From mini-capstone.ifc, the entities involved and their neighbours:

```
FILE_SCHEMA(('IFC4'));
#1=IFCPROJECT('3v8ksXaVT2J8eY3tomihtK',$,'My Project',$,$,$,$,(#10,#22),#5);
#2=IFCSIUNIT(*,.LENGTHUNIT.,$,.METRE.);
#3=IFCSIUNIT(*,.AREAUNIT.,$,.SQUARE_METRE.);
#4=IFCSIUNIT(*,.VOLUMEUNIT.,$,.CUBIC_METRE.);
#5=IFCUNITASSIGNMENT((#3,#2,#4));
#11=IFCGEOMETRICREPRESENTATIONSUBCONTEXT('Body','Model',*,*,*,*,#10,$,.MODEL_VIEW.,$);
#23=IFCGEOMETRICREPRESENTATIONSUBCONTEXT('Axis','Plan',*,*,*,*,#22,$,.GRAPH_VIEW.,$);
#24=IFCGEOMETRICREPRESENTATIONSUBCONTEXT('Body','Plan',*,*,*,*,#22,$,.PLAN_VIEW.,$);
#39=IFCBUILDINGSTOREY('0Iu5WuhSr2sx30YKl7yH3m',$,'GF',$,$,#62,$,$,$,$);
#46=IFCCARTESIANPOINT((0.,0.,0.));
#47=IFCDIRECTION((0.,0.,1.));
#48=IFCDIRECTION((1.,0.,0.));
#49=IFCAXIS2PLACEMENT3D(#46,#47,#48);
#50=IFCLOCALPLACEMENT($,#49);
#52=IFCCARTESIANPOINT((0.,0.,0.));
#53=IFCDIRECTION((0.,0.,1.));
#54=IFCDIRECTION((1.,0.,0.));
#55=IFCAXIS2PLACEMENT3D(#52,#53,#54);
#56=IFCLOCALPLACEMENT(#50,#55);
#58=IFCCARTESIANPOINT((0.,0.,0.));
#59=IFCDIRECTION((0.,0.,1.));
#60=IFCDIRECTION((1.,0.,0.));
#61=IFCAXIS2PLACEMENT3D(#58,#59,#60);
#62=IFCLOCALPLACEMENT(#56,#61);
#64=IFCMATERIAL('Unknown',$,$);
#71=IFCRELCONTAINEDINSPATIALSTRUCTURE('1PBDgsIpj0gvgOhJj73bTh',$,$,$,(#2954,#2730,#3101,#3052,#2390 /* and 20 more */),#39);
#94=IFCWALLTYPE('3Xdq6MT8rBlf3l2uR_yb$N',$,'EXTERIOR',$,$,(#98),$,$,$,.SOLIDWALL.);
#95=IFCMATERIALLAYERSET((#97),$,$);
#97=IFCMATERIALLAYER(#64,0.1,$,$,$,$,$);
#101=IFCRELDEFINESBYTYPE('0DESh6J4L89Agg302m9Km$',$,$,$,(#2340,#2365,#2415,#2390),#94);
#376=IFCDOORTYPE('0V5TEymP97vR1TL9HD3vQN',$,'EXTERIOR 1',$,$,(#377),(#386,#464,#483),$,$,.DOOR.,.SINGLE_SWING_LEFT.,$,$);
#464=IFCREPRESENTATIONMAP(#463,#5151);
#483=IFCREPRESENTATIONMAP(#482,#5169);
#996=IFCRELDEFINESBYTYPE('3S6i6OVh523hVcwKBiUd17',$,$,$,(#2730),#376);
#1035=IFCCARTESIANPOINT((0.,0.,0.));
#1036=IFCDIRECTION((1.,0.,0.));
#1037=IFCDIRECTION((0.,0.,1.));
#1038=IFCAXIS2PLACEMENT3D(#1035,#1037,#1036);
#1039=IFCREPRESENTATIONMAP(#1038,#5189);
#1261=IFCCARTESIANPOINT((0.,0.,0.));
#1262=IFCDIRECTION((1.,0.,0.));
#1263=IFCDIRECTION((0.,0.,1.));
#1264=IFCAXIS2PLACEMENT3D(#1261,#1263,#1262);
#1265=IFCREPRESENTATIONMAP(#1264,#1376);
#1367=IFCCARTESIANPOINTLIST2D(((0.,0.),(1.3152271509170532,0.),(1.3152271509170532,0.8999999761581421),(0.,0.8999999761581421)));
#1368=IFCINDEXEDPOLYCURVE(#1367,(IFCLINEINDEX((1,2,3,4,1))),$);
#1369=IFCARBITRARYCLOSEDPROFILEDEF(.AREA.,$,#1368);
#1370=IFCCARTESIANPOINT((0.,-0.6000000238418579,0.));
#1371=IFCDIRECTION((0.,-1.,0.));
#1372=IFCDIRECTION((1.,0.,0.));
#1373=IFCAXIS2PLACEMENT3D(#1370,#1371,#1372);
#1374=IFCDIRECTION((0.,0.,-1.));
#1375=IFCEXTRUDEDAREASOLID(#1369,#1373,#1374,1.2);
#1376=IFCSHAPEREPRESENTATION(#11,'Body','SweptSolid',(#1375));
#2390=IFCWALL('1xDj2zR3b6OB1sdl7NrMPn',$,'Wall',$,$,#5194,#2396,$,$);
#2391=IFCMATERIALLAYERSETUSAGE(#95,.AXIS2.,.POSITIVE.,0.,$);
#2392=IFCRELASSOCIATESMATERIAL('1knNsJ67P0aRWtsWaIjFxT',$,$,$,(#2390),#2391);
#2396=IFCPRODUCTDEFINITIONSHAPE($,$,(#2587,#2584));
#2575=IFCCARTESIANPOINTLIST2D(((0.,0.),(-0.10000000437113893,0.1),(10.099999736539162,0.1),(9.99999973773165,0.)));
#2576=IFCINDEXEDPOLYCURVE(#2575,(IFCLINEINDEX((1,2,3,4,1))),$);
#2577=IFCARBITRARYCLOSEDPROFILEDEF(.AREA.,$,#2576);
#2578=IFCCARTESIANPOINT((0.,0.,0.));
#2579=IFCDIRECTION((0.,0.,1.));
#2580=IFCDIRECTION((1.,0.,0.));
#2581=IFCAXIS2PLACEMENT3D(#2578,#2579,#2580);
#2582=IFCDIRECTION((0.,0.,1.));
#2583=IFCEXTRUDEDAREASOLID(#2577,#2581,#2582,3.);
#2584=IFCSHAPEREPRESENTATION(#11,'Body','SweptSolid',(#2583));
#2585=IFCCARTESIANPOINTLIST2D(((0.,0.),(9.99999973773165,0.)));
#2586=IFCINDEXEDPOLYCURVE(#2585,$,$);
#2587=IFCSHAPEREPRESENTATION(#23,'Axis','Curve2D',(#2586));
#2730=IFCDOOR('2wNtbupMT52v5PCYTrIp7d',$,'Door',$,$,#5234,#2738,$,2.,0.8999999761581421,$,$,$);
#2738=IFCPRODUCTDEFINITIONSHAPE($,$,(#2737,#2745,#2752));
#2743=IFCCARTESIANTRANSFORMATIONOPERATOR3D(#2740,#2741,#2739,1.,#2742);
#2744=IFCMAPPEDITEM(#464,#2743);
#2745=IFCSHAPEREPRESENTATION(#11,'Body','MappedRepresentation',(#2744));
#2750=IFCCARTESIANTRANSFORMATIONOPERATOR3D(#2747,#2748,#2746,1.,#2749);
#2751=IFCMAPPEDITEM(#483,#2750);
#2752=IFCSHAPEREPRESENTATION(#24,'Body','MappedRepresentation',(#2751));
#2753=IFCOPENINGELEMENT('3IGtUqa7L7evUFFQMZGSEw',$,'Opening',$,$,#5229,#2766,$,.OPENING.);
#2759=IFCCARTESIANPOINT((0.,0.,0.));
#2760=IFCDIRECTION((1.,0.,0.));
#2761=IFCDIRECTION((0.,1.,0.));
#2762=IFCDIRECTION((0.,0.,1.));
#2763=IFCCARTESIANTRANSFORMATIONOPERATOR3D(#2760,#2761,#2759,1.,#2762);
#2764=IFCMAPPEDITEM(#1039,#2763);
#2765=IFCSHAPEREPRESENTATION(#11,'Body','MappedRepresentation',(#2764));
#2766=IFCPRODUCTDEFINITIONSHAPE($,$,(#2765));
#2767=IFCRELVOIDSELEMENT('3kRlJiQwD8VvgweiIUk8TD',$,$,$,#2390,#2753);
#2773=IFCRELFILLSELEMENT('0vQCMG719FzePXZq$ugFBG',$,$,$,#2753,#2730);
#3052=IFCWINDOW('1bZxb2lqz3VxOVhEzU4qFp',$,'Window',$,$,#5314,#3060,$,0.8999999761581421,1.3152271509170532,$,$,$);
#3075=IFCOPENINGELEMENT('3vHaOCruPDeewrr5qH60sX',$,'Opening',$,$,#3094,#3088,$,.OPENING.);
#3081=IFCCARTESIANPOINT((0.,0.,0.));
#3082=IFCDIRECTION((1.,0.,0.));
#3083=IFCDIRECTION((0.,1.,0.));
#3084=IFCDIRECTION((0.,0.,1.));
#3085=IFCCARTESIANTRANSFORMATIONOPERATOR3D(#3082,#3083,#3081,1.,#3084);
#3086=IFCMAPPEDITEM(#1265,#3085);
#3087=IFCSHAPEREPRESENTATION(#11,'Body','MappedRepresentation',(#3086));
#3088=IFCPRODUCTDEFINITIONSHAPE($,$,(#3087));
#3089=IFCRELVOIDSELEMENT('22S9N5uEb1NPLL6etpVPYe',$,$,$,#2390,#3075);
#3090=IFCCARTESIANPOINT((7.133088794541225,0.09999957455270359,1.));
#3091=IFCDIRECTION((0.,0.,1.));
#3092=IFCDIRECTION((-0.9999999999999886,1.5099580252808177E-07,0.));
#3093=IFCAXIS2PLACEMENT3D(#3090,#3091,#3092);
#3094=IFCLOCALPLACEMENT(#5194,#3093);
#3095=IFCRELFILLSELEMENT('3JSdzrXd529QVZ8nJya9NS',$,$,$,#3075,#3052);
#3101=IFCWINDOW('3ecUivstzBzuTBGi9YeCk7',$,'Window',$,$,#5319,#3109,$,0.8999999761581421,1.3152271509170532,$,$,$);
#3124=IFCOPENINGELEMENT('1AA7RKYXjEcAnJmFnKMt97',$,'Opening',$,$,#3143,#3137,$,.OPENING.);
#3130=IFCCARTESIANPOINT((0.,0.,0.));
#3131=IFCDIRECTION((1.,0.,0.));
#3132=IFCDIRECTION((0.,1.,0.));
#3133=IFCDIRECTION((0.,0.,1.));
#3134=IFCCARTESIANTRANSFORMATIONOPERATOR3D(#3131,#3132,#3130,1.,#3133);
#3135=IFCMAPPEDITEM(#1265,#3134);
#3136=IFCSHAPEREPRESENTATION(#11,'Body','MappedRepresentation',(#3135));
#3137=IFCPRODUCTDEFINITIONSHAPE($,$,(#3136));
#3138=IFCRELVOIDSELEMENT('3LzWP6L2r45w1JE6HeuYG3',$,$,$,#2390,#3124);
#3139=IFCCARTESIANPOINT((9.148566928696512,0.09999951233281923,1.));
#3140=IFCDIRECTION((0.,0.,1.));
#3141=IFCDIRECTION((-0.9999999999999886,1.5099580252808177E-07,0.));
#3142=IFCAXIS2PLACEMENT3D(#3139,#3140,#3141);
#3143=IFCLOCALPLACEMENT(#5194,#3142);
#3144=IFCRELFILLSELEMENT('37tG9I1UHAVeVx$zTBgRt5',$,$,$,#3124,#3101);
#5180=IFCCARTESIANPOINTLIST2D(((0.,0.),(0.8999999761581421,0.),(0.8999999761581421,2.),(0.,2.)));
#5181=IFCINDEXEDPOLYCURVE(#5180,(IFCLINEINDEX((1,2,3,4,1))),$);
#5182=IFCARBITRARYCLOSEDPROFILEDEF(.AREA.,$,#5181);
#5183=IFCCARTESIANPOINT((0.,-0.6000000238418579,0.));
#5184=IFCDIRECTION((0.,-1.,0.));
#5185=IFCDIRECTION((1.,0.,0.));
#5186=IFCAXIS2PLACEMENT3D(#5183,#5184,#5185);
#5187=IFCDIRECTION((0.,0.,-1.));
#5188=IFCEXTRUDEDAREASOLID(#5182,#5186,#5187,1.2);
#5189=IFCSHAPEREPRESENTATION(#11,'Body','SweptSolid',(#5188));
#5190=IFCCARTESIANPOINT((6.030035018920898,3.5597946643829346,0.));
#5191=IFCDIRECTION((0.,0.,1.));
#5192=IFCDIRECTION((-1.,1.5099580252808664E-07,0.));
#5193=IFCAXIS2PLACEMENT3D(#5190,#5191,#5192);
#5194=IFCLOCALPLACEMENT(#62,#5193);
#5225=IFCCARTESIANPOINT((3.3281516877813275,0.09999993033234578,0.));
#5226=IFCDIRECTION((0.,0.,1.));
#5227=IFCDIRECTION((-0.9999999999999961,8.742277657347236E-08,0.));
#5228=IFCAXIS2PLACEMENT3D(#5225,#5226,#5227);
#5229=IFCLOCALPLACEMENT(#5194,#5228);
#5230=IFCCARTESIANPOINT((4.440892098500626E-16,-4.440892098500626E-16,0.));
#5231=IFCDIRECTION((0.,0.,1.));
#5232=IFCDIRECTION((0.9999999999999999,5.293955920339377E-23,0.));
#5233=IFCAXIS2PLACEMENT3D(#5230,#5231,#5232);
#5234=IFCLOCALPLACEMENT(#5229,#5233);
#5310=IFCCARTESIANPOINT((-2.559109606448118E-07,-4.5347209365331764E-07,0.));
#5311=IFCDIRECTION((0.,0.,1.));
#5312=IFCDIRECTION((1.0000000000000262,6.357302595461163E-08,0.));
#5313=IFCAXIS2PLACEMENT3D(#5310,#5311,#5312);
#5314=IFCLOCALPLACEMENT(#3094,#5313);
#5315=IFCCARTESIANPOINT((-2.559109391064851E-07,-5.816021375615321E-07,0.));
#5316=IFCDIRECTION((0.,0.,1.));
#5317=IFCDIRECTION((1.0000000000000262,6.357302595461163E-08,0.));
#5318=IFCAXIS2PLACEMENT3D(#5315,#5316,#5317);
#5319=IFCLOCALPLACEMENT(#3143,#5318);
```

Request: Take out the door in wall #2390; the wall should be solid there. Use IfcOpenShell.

```python
import ifcopenshell
import ifcopenshell.api.feature
import ifcopenshell.api.root
import ifcopenshell.geom
import ifcopenshell.util.shape

model = ifcopenshell.open("mini-capstone.ifc")
settings = ifcopenshell.geom.settings()


def volume(element):
    """Net volume in cubic metres, openings subtracted."""
    shape = ifcopenshell.geom.create_shape(settings, element)
    return ifcopenshell.util.shape.get_volume(shape.geometry)


door = model.by_guid("2wNtbupMT52v5PCYTrIp7d")
opening = door.FillsVoids[0].RelatingOpeningElement
wall = opening.VoidsElements[0].RelatingBuildingElement
before = volume(wall)

ifcopenshell.api.root.remove_product(model, product=door)
ifcopenshell.api.feature.remove_feature(model, feature=opening)

after = volume(wall)

print(f"wall volume {before:.3f} -> {after:.3f} m3")

model.write("mini-capstone_edited.ifc")
```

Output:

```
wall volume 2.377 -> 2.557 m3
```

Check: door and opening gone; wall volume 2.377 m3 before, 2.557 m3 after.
